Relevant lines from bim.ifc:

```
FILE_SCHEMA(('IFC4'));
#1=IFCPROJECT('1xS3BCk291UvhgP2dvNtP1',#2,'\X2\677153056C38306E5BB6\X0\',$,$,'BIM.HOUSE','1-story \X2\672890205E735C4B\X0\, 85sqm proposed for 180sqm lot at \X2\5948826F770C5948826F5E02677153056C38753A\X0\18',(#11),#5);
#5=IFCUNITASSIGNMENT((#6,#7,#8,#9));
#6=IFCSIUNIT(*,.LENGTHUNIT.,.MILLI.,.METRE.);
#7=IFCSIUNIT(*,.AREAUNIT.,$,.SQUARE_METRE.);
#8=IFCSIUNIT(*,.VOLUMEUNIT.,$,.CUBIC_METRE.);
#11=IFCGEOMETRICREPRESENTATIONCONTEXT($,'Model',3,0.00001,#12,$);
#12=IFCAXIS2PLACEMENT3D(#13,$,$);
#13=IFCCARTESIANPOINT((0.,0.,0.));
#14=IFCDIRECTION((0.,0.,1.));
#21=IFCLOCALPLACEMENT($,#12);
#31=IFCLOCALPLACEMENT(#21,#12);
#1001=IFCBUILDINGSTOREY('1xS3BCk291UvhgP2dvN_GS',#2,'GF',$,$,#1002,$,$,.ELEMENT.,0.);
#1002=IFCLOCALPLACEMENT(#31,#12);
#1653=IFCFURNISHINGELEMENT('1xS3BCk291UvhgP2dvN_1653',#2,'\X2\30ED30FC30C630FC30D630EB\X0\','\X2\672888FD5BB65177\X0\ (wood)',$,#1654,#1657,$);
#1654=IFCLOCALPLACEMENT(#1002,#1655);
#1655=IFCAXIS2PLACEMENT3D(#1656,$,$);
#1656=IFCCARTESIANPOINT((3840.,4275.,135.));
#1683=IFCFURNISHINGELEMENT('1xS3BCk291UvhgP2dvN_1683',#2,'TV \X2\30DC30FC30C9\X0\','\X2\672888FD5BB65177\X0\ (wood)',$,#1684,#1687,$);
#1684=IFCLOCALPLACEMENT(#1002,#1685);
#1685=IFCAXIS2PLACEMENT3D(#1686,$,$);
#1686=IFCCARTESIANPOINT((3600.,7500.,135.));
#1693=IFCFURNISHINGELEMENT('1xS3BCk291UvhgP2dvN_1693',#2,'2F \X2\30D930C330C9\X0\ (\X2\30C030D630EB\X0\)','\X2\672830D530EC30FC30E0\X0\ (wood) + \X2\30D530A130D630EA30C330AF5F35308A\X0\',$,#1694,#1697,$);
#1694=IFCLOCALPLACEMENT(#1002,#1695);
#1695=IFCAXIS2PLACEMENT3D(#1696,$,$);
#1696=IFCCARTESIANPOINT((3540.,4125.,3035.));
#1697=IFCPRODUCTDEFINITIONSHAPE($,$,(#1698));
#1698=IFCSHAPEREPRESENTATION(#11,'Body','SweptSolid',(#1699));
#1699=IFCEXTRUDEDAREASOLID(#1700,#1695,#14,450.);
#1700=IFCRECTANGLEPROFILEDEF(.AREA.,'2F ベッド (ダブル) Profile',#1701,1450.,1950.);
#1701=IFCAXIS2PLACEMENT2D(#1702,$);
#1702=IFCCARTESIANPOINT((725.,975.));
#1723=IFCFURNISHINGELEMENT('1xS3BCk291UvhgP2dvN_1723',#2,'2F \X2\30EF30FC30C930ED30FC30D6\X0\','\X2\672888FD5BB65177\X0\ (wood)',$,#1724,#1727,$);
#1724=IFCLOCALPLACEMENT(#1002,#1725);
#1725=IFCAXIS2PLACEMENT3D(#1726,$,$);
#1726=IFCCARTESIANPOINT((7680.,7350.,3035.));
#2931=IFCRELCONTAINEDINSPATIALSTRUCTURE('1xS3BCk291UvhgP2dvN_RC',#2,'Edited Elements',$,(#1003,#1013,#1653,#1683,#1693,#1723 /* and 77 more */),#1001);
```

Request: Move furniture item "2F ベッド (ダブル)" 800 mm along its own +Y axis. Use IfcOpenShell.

```python
import ifcopenshell
import ifcopenshell.api.geometry
import ifcopenshell.util.placement

model = ifcopenshell.open("bim.ifc")

item = model.by_guid("1xS3BCk291UvhgP2dvN_1693")
matrix = ifcopenshell.util.placement.get_local_placement(item.ObjectPlacement)
matrix[:3, 3] += matrix[:3, 1] * 800.0
ifcopenshell.api.geometry.edit_object_placement(model, product=item, matrix=matrix, is_si=False)

print(ifcopenshell.util.placement.get_local_placement(item.ObjectPlacement).round(3) + 0.0)

model.write("bim_updated.ifc")
```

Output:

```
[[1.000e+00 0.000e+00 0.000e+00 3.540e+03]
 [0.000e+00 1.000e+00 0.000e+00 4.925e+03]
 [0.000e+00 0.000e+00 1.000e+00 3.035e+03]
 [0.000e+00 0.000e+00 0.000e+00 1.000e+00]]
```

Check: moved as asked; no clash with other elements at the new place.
